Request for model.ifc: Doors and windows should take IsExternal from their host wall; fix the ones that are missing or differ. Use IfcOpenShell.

First a look at what the model holds.

```python
import ifcopenshell
import ifcopenshell.util.element

model = ifcopenshell.open("model.ifc")
print(model.schema)
seen = {}
for e in model.by_type("IfcDoor") + model.by_type("IfcWindow"):
    if not e.FillsVoids:
        continue
    host = e.FillsVoids[0].RelatingOpeningElement.VoidsElements[0].RelatingBuildingElement
    own = ifcopenshell.util.element.get_pset(e, f"Pset_{e.is_a()[3:].removesuffix('StandardCase')}Common", "IsExternal")
    wall = ifcopenshell.util.element.get_pset(host, "Pset_WallCommon", "IsExternal")
    seen[e.is_a(), own, wall] = seen.get((e.is_a(), own, wall), 0) + 1
for (cls, own, wall), count in sorted(seen.items(), key=str):
    print(count, cls, "IsExternal:", own, "| host wall:", wall)
```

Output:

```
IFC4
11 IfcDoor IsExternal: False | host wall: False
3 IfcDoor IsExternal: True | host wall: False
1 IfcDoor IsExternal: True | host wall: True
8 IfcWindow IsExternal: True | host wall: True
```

```python
import ifcopenshell
import ifcopenshell.api.pset
import ifcopenshell.util.element

model = ifcopenshell.open("model.ifc")

count = 0
for ifc_class, pset_name in (("IfcDoor", "Pset_DoorCommon"), ("IfcWindow", "Pset_WindowCommon")):
    for e in model.by_type(ifc_class):
        if not e.FillsVoids:
            continue
        host = e.FillsVoids[0].RelatingOpeningElement.VoidsElements[0].RelatingBuildingElement
        external = ifcopenshell.util.element.get_pset(host, "Pset_WallCommon", "IsExternal")
        if external is None or ifcopenshell.util.element.get_pset(e, pset_name, "IsExternal") == external:
            continue
        pset = ifcopenshell.api.pset.add_pset(model, product=e, name=pset_name)
        ifcopenshell.api.pset.edit_pset(model, pset=pset, properties={"IsExternal": external})
        count += 1

print(count, "updated")

model.write("model_v2.ifc")
```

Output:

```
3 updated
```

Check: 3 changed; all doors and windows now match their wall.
